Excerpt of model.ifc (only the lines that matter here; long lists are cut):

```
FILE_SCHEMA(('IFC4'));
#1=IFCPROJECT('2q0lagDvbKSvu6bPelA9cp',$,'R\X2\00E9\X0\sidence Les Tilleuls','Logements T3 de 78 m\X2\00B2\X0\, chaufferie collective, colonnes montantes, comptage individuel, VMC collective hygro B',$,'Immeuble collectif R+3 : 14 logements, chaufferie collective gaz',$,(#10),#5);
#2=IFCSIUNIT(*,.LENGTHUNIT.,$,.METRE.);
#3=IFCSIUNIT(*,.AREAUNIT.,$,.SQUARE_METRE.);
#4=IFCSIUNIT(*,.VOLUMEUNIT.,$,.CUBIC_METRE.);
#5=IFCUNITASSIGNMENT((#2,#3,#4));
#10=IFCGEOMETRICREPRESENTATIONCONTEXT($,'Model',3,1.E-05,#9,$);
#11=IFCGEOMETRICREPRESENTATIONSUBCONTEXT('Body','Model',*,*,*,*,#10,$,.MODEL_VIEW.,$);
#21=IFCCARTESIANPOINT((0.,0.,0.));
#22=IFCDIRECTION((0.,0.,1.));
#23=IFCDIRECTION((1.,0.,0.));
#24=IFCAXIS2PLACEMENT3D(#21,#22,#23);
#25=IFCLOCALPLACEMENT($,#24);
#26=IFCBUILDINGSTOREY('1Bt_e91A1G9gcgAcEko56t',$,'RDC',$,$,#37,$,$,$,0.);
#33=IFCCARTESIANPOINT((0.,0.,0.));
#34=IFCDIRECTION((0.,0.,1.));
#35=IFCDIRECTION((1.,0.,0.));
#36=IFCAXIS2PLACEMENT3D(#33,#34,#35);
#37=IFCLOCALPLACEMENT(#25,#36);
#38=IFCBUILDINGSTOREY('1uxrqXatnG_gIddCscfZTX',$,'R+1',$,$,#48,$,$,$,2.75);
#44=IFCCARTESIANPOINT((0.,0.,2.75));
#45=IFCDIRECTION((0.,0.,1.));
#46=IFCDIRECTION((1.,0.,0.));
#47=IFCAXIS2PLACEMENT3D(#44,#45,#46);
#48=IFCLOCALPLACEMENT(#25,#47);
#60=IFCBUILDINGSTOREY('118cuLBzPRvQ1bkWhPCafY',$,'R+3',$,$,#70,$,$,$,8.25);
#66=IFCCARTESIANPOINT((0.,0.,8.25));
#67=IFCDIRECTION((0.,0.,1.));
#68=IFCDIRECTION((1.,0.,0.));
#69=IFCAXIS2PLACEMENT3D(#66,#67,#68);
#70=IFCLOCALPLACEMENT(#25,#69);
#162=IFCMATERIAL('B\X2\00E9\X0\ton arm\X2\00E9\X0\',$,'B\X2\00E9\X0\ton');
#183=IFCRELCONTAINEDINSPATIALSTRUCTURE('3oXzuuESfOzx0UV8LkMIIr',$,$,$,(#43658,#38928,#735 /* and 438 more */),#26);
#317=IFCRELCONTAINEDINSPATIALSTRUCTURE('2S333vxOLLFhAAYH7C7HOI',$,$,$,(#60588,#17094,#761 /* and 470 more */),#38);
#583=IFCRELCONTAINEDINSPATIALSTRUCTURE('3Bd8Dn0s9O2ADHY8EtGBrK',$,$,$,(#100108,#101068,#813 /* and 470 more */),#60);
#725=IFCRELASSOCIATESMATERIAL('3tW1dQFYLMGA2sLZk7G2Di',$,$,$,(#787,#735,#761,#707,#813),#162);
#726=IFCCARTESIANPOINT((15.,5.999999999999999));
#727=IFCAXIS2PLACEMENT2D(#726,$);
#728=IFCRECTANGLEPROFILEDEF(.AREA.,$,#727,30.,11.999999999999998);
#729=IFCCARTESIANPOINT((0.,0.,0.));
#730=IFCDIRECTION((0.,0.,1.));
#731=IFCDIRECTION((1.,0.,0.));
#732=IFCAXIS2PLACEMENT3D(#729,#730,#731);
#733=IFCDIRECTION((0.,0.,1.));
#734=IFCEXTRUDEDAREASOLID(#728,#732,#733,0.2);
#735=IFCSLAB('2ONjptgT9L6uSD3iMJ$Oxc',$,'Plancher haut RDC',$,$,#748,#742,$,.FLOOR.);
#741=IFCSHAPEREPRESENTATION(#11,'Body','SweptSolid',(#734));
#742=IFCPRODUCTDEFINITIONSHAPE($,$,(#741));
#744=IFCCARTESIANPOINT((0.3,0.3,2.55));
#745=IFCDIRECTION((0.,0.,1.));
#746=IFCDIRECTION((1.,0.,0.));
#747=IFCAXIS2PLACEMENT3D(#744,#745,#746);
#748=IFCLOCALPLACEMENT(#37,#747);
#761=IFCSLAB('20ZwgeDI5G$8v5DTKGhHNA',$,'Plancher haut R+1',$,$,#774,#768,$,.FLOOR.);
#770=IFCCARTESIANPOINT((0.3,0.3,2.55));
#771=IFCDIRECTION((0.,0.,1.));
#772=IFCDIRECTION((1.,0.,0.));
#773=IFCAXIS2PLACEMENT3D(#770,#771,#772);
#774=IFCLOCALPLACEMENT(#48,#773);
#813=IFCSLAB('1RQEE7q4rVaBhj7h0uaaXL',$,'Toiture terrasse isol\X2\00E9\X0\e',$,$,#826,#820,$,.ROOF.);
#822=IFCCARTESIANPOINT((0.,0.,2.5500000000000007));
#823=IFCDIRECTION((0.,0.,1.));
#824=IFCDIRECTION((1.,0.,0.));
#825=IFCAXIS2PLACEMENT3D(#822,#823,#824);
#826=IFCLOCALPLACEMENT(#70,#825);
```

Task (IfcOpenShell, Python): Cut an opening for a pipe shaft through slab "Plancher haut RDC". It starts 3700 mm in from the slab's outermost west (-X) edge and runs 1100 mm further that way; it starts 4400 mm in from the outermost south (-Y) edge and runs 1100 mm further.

```python
import numpy as np
import ifcopenshell
import ifcopenshell.api.feature
import ifcopenshell.api.geometry
import ifcopenshell.api.root
import ifcopenshell.geom
import ifcopenshell.util.placement
import ifcopenshell.util.representation
import ifcopenshell.util.shape
import ifcopenshell.util.unit

model = ifcopenshell.open("model.ifc")
unit_scale = ifcopenshell.util.unit.calculate_unit_scale(model)
settings = ifcopenshell.geom.settings()


def volume(element):
    """Net volume in cubic metres, openings subtracted."""
    shape = ifcopenshell.geom.create_shape(settings, element)
    return ifcopenshell.util.shape.get_volume(shape.geometry)


slab = model.by_id(735)
before = volume(slab)

# Extent in the slab's own axes, in metres. The edges named are its -X and -Y sides.
slab_shape = ifcopenshell.geom.create_shape(settings, slab)
vertices = ifcopenshell.util.shape.get_vertices(slab_shape.geometry)
x_min, y_min, bottom = vertices.min(axis=0)
top = vertices[:, 2].max()

opening = ifcopenshell.api.root.create_entity(model, ifc_class="IfcOpeningElement", name="Pipe shaft opening", predefined_type="OPENING")
context = ifcopenshell.util.representation.get_context(model, "Model", "Body", "MODEL_VIEW")
width, depth = 1.1, 1.1
outline = [(0.0, 0.0), (width, 0.0), (width, depth), (0.0, depth), (0.0, 0.0)]
# Overshoot both faces by 50 mm so the cut is clean.
shape = ifcopenshell.api.geometry.add_slab_representation(
    model, context=context, depth=top - bottom + 0.1, polyline=outline
)
ifcopenshell.api.geometry.assign_representation(model, product=opening, representation=shape)

matrix = ifcopenshell.util.placement.get_local_placement(slab.ObjectPlacement)
matrix[:, 3] = matrix @ np.append(np.array([x_min + 3.7, y_min + 4.4, bottom - 0.05]) / unit_scale, 1.0)
ifcopenshell.api.geometry.edit_object_placement(model, product=opening, matrix=matrix, is_si=False)
ifcopenshell.api.feature.add_feature(model, feature=opening, element=slab)

after = volume(slab)

print(f"slab volume {before:.3f} -> {after:.3f} m3")

model.write("model_updated.ifc")
```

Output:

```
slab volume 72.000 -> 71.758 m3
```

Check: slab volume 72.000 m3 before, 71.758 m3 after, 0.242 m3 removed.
